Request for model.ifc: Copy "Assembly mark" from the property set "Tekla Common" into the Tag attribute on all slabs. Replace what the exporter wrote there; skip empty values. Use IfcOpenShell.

First a look at what the model holds.

```python
import ifcopenshell
import ifcopenshell.util.element

model = ifcopenshell.open("model.ifc")
print(model.schema)
slabs = model.by_type("IfcSlab")
print(len(slabs), "slabs")
for e in slabs[:8]:
    source = ifcopenshell.util.element.get_pset(e, "Tekla Common", "Assembly mark")
    target = e.Tag
    print(e.id(), repr(source), repr(target), sep=" | ")
```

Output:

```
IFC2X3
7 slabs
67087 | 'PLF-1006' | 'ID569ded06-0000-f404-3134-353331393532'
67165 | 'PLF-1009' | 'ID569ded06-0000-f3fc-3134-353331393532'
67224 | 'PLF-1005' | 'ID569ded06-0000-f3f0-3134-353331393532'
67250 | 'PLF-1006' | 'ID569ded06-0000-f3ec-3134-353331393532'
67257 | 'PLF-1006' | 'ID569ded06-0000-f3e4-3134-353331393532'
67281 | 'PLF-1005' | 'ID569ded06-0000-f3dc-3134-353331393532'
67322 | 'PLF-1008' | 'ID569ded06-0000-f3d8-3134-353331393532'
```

```python
import ifcopenshell
import ifcopenshell.util.element

model = ifcopenshell.open("model.ifc")

count = 0
for e in model.by_type("IfcSlab"):
    value = ifcopenshell.util.element.get_pset(e, "Tekla Common", "Assembly mark")
    current = e.Tag
    if not value or not value.strip() or current == value:
        continue
    e.Tag = value
    count += 1

print(count, "slabs updated")

model.write("model_rev.ifc")
```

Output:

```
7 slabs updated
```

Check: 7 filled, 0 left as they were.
